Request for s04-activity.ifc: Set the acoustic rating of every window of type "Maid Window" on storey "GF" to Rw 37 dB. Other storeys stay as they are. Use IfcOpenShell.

First a look at what the model holds.

```python
import ifcopenshell
import ifcopenshell.util.element

model = ifcopenshell.open("s04-activity.ifc")
print(model.schema)
storey = next(s for s in model.by_type("IfcBuildingStorey") if s.Name == "GF")
windows = [e for e in ifcopenshell.util.element.get_decomposition(storey) if e.is_a("IfcWindow")]
seen = {}
for e in windows:
    element_type = ifcopenshell.util.element.get_type(e)
    key = (element_type.Name if element_type != e and element_type else None, ifcopenshell.util.element.get_pset(e, "Pset_WindowCommon", "AcousticRating"))
    seen[key] = seen.get(key, 0) + 1
for (name, value), count in sorted(seen.items(), key=str):
    print(count, "x", name, "|", value)
```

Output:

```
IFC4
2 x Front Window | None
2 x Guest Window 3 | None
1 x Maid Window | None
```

```python
import ifcopenshell
import ifcopenshell.api.pset
import ifcopenshell.util.element

model = ifcopenshell.open("s04-activity.ifc")

storey = next(s for s in model.by_type("IfcBuildingStorey") if s.Name == "GF")
windows = [e for e in ifcopenshell.util.element.get_decomposition(storey) if e.is_a("IfcWindow")]

count = 0
for e in windows:
    element_type = ifcopenshell.util.element.get_type(e)
    if element_type in (None, e) or element_type.Name != "Maid Window":
        continue
    # add_pset returns the element's existing set when there is one.
    pset = ifcopenshell.api.pset.add_pset(model, product=e, name="Pset_WindowCommon")
    ifcopenshell.api.pset.edit_pset(model, pset=pset, properties={"AcousticRating": "Rw 37 dB"})
    count += 1

print(count, "windows updated")

model.write("s04-activity_updated.ifc")
```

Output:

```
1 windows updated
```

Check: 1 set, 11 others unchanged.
